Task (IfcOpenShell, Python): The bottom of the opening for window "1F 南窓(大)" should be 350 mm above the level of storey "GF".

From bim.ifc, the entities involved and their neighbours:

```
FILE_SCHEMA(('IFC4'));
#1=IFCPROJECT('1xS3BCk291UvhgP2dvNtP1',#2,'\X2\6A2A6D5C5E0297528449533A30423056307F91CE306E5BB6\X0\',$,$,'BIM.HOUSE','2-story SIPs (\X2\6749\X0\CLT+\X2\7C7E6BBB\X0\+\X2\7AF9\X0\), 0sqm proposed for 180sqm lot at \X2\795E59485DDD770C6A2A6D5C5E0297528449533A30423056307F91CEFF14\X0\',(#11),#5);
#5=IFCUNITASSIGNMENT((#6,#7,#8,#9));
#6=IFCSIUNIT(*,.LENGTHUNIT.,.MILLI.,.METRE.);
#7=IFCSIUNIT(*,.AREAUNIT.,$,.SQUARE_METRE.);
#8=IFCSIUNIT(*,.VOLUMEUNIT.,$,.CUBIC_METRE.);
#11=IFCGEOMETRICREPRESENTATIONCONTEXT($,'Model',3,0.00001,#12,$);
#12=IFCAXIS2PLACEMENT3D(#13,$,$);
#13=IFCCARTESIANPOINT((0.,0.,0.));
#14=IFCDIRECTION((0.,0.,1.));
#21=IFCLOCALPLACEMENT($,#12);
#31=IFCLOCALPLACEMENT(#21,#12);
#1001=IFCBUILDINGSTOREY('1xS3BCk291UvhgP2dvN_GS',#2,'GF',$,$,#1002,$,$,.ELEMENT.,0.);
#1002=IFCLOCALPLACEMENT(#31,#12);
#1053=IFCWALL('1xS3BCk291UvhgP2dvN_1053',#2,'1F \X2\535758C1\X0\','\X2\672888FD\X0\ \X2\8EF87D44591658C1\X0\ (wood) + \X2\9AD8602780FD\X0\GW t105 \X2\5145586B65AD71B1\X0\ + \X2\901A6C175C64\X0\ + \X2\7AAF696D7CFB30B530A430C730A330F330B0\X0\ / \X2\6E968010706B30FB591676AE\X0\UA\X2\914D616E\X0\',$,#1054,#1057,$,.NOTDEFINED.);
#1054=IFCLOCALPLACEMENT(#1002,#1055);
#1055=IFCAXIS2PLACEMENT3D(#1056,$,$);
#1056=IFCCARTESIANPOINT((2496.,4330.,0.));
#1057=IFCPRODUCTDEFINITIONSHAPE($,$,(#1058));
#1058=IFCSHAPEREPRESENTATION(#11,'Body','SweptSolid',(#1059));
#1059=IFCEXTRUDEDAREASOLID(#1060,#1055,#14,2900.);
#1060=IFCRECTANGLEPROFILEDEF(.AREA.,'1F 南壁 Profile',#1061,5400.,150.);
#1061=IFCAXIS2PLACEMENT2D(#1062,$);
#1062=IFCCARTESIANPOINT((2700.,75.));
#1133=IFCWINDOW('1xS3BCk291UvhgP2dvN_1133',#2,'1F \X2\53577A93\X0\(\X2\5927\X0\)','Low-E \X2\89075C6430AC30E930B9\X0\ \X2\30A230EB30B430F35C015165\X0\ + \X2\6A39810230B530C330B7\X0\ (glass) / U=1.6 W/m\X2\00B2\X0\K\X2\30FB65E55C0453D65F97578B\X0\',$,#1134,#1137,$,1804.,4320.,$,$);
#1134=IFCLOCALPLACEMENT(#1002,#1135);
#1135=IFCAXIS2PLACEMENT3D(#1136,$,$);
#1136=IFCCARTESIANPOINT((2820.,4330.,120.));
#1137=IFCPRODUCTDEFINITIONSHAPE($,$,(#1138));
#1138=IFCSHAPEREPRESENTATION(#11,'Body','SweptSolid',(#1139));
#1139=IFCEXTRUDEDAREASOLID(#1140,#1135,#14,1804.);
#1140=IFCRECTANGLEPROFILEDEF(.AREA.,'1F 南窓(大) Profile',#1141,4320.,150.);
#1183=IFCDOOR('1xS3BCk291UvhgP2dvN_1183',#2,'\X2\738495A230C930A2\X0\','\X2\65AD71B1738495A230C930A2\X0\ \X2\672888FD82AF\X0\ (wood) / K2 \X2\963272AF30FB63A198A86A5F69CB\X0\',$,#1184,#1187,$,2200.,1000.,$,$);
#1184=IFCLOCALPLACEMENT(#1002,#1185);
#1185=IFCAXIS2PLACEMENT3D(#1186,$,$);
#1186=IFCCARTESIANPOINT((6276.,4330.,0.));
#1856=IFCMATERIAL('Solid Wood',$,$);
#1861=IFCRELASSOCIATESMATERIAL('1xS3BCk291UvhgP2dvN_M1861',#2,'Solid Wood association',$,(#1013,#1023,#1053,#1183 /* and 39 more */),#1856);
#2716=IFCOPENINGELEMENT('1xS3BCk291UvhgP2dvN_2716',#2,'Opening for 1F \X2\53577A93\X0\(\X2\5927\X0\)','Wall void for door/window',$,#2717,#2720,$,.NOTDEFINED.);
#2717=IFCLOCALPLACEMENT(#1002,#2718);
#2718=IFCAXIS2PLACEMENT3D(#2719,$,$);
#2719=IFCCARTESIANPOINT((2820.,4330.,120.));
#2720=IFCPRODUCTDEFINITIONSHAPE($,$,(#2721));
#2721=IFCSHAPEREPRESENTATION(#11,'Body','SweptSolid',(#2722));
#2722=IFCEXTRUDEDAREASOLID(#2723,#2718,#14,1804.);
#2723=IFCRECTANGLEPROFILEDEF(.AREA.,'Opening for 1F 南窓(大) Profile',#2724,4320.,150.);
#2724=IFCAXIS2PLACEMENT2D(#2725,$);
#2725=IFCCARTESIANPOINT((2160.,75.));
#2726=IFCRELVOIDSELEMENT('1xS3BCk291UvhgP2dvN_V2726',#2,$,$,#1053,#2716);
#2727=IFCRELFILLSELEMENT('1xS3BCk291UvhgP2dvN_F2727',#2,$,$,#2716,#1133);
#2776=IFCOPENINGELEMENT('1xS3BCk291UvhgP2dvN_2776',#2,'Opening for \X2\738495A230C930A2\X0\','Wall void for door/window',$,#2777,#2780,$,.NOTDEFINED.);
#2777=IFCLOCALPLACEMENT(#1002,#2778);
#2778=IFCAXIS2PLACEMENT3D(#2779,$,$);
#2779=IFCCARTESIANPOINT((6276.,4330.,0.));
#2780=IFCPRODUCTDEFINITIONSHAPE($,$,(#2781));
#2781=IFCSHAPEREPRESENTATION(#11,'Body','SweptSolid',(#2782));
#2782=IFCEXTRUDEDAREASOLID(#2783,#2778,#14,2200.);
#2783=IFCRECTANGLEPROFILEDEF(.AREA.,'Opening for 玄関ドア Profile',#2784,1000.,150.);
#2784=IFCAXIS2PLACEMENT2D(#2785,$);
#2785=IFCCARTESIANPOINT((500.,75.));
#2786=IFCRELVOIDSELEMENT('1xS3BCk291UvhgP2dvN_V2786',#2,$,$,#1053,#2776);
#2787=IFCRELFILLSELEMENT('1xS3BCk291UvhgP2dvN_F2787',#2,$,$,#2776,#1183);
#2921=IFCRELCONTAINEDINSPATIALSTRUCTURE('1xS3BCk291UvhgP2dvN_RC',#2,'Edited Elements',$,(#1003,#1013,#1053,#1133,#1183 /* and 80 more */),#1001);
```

```python
import numpy as np
import ifcopenshell
import ifcopenshell.api.geometry
import ifcopenshell.geom
import ifcopenshell.util.element
import ifcopenshell.util.placement
import ifcopenshell.util.shape
import ifcopenshell.util.unit

model = ifcopenshell.open("bim.ifc")
unit_scale = ifcopenshell.util.unit.calculate_unit_scale(model)

window = model.by_guid("1xS3BCk291UvhgP2dvN_1133")
opening = window.FillsVoids[0].RelatingOpeningElement
storey = ifcopenshell.util.element.get_container(window, ifc_class="IfcBuildingStorey")
level = ifcopenshell.util.placement.get_local_placement(storey.ObjectPlacement)[2, 3]

# The opening's origin need not be at the sill, so measure its lowest point.
shape = ifcopenshell.geom.create_shape(ifcopenshell.geom.settings(), opening)
bottom = ifcopenshell.util.shape.get_shape_bottom_elevation(shape, shape.geometry) / unit_scale
dz = level + 350.0 - bottom

shift = np.array([0.0, 0.0, dz])
# The window is not placed relative to its opening, so move both.
for product in (opening, window):
    matrix = ifcopenshell.util.placement.get_local_placement(product.ObjectPlacement)
    matrix[:3, 3] += shift
    ifcopenshell.api.geometry.edit_object_placement(model, product=product, matrix=matrix, is_si=False)

print(f"moved by {dz * unit_scale:+.3f} m")

model.write("bim_edited.ifc")
```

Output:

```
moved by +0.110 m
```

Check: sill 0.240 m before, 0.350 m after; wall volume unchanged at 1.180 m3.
